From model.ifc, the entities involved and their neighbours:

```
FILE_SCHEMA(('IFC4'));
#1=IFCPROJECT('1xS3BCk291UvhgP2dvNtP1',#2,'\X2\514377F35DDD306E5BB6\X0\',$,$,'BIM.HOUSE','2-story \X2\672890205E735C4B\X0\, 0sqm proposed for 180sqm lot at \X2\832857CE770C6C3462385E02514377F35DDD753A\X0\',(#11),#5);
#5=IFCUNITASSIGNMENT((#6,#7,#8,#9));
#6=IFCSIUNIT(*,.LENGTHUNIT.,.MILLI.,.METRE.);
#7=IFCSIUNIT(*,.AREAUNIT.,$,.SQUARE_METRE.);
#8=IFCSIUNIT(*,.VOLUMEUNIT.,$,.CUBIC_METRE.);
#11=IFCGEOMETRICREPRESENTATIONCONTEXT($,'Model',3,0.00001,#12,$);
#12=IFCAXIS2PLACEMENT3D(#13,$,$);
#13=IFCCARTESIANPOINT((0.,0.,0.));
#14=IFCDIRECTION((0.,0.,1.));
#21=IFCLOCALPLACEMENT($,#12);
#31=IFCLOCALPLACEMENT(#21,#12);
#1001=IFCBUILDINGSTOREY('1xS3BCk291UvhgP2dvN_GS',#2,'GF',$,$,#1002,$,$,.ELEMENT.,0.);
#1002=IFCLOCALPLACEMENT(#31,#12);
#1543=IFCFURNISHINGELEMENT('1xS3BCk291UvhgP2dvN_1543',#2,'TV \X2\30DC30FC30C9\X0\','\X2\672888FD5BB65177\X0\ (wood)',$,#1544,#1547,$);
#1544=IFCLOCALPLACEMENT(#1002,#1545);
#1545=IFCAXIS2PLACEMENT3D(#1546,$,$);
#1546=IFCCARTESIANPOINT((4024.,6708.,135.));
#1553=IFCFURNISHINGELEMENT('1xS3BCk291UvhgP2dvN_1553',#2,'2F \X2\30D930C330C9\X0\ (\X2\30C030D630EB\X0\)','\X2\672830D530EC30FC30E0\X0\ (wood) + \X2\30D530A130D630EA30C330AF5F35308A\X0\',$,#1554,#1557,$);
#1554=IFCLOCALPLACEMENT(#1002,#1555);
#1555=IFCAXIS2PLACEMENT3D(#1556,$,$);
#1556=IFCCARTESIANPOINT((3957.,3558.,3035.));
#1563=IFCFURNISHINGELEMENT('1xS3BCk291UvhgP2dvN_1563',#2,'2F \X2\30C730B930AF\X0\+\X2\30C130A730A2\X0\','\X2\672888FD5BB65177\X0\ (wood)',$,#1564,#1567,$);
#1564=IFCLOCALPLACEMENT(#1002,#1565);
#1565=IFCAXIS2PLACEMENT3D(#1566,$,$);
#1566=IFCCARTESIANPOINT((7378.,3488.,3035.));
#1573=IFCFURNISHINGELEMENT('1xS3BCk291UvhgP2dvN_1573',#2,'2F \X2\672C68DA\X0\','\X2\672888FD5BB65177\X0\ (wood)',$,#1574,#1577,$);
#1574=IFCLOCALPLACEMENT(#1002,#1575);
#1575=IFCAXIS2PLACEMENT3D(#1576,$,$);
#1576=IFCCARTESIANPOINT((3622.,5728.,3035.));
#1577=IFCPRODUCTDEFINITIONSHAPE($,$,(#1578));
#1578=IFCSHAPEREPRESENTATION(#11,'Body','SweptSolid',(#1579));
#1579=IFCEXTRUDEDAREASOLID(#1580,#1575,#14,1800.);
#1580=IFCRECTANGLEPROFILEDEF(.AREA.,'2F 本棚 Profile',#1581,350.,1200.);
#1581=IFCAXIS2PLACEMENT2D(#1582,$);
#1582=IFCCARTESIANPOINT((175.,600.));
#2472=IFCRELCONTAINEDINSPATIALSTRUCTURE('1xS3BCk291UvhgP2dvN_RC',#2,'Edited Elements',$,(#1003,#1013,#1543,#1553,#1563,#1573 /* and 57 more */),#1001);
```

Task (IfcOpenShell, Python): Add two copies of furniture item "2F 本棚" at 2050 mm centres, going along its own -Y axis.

```python
import ifcopenshell
import ifcopenshell.api.geometry
import ifcopenshell.api.root
import ifcopenshell.util.element
import ifcopenshell.util.placement
import ifcopenshell.util.unit

model = ifcopenshell.open("model.ifc")
unit_scale = ifcopenshell.util.unit.calculate_unit_scale(model)


def reuse_history(source, copy):
    """copy_class also copies each property set's owner history, people and application; keep the originals."""
    for rel in copy.IsDefinedBy:
        if rel.is_a("IfcRelDefinesByProperties") and (history := rel.RelatingPropertyDefinition.OwnerHistory):
            rel.RelatingPropertyDefinition.OwnerHistory = source.OwnerHistory
            ifcopenshell.util.element.remove_deep2(model, history)


source = model.by_guid("1xS3BCk291UvhgP2dvN_1573")
base = ifcopenshell.util.placement.get_local_placement(source.ObjectPlacement)
step = -base[:3, 1] * 2.05 / unit_scale

for i in range(1, 3):
    copy = ifcopenshell.api.root.copy_class(model, product=source)
    copy.Representation = ifcopenshell.util.element.copy_deep(
        model, source.Representation, exclude=["IfcGeometricRepresentationContext", "IfcRepresentationMap"]
    )
    reuse_history(source, copy)
    matrix = base.copy()
    matrix[:3, 3] += i * step
    print("added at", matrix[:3, 3].round(3) + 0.0)
    ifcopenshell.api.geometry.edit_object_placement(model, product=copy, matrix=matrix, is_si=False)

model.write("model-out.ifc")
```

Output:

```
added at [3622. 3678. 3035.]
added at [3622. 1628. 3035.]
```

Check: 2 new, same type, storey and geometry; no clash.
